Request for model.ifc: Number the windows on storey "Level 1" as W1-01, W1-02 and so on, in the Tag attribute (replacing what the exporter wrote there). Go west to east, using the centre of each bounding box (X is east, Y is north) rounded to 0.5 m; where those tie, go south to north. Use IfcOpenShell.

First a look at what the model holds.

```python
import ifcopenshell
import ifcopenshell.util.element
import ifcopenshell.util.placement

model = ifcopenshell.open("model.ifc")
print(model.schema)
storey = next(s for s in model.by_type("IfcBuildingStorey") if s.Name == "Level 1")
windows = [e for e in ifcopenshell.util.element.get_decomposition(storey) if e.is_a("IfcWindow")]
for e in sorted(windows, key=lambda e: e.id()):
    origin = ifcopenshell.util.placement.get_local_placement(e.ObjectPlacement)[:3, 3]
    print(e.id(), e.Tag, e.Name, origin.round(2) + 0.0, sep=" | ")
```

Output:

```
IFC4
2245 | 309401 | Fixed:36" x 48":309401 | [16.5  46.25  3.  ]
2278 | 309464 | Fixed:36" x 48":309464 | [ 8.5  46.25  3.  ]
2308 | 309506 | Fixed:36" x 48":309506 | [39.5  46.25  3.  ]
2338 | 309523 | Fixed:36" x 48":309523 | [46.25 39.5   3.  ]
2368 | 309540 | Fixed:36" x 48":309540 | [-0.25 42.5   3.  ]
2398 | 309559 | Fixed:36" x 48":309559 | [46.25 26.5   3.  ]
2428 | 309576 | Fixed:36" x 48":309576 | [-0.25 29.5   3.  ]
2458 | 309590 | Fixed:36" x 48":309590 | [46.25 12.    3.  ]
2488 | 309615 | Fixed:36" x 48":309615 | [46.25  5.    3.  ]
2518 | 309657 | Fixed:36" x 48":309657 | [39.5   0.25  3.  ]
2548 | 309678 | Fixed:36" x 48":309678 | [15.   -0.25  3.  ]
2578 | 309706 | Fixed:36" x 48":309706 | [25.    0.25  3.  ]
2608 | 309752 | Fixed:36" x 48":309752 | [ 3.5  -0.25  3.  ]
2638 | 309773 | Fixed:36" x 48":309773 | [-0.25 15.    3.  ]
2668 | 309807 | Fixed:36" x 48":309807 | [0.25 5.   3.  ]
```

```python
import ifcopenshell
import ifcopenshell.geom
import ifcopenshell.util.element
import ifcopenshell.util.shape

model = ifcopenshell.open("model.ifc")
settings = ifcopenshell.geom.settings()
settings.set("use-world-coords", True)


def centre(element):
    shape = ifcopenshell.geom.create_shape(settings, element)
    return ifcopenshell.util.shape.get_bbox_centroid(shape.geometry)


storey = next(s for s in model.by_type("IfcBuildingStorey") if s.Name == "Level 1")
windows = [e for e in ifcopenshell.util.element.get_decomposition(storey) if e.is_a("IfcWindow")]

# Insertion points can sit at a corner or the storey origin, so sort by the geometry (in metres).
centres = {e: centre(e) for e in windows}
windows.sort(key=lambda e: (round(centres[e][0] / 0.5), centres[e][1]))

for i, e in enumerate(windows, start=1):
    number = f"W1-{i:02d}"
    e.Tag = number
    print(e.id(), number)

model.write("model_updated.ifc")
```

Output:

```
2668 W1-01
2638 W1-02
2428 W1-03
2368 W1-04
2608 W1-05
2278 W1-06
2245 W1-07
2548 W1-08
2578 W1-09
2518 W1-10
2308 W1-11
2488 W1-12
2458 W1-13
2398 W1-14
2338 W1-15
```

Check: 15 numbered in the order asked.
